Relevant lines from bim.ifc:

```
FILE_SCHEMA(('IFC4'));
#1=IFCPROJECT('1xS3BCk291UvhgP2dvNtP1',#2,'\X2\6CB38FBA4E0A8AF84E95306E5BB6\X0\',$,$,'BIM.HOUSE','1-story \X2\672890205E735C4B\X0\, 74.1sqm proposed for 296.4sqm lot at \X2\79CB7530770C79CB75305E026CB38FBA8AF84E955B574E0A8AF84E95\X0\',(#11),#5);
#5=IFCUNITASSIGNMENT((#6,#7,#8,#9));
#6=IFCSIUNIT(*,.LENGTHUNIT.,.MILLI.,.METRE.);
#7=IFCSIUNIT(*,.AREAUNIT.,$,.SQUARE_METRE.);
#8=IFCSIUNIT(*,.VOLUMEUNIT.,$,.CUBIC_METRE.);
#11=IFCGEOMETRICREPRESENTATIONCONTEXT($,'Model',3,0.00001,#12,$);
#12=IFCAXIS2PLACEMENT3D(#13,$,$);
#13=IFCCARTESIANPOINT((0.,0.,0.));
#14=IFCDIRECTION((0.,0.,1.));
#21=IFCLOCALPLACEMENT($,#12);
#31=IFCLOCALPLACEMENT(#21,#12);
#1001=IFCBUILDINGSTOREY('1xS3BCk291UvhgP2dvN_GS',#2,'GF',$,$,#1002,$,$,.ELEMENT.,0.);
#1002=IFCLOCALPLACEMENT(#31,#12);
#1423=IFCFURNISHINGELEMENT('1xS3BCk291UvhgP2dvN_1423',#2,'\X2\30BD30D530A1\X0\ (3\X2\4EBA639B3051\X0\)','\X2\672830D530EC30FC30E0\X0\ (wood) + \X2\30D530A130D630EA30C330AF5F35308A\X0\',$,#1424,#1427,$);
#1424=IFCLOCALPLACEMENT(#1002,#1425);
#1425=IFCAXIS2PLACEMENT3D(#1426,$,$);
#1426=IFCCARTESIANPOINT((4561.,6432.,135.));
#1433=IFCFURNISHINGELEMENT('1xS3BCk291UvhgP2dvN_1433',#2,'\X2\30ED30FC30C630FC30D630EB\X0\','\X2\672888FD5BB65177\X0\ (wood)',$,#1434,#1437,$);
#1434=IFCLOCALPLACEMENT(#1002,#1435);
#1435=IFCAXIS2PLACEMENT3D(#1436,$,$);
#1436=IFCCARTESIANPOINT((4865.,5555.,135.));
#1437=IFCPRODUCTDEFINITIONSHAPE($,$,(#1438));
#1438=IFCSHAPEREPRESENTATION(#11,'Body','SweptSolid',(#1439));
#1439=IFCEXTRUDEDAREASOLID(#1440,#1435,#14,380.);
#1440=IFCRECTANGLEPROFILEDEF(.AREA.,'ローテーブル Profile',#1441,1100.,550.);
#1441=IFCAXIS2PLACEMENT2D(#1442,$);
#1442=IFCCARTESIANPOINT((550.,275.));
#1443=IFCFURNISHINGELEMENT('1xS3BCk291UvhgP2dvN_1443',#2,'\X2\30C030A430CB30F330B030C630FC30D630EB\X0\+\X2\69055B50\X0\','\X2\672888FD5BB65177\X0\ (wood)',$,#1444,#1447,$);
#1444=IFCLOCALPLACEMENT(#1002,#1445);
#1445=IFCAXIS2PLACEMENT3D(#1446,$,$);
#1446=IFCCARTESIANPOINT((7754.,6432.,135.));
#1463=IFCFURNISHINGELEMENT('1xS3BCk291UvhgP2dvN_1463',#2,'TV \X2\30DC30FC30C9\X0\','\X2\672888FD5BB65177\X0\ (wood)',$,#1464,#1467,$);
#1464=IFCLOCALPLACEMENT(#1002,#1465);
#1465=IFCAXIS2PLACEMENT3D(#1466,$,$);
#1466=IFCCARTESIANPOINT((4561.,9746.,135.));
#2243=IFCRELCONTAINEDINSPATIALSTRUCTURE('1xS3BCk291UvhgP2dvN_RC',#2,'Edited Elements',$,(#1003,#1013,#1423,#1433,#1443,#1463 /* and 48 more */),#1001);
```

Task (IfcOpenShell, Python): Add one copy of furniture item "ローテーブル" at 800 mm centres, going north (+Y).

```python
import numpy as np
import ifcopenshell
import ifcopenshell.api.geometry
import ifcopenshell.api.root
import ifcopenshell.util.element
import ifcopenshell.util.placement

model = ifcopenshell.open("bim.ifc")


def reuse_history(source, copy):
    """copy_class also copies each property set's owner history, people and application; keep the originals."""
    for rel in copy.IsDefinedBy:
        if rel.is_a("IfcRelDefinesByProperties") and (history := rel.RelatingPropertyDefinition.OwnerHistory):
            rel.RelatingPropertyDefinition.OwnerHistory = source.OwnerHistory
            ifcopenshell.util.element.remove_deep2(model, history)


source = model.by_id(1433)
base = ifcopenshell.util.placement.get_local_placement(source.ObjectPlacement)
step = np.array([0.0, 1.0, 0.0]) * 800.0

for i in range(1, 2):
    copy = ifcopenshell.api.root.copy_class(model, product=source)
    copy.Representation = ifcopenshell.util.element.copy_deep(
        model, source.Representation, exclude=["IfcGeometricRepresentationContext", "IfcRepresentationMap"]
    )
    reuse_history(source, copy)
    matrix = base.copy()
    matrix[:3, 3] += i * step
    print("added at", matrix[:3, 3].round(3) + 0.0)
    ifcopenshell.api.geometry.edit_object_placement(model, product=copy, matrix=matrix, is_si=False)

model.write("bim_rev.ifc")
```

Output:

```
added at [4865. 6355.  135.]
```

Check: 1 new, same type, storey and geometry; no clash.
